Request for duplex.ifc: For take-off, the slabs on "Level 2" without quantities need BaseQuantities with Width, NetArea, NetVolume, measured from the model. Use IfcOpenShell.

First a look at what the model holds.

```python
import ifcopenshell
import ifcopenshell.util.element
import ifcopenshell.util.unit

model = ifcopenshell.open("duplex.ifc")
print(model.schema)
for unit_type in ("LENGTHUNIT", "AREAUNIT", "VOLUMEUNIT"):
    print(unit_type, ifcopenshell.util.unit.calculate_unit_scale(model, unit_type))
storey = next(s for s in model.by_type("IfcBuildingStorey") if s.Name == "Level 2")
slabs = [e for e in ifcopenshell.util.element.get_decomposition(storey) if e.is_a("IfcSlab")]
for e in sorted(slabs, key=lambda e: e.id()):
    print(e.id(), e.is_a(), e.Name, list(ifcopenshell.util.element.get_psets(e, qtos_only=True)), sep=" | ")
```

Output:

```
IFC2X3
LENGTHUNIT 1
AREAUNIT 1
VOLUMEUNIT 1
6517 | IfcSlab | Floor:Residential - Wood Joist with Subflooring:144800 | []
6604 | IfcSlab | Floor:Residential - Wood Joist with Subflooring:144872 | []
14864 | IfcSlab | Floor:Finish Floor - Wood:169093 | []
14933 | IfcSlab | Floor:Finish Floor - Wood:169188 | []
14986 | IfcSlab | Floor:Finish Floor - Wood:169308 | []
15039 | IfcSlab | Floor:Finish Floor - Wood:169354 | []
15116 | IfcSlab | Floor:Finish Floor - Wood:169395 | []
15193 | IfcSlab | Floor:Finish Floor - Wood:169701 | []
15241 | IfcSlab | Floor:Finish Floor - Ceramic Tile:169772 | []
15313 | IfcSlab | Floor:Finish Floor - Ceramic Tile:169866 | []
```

```python
import ifcopenshell
import ifcopenshell.api.pset
import ifcopenshell.geom
import ifcopenshell.util.element
import ifcopenshell.util.shape
import ifcopenshell.util.unit

model = ifcopenshell.open("duplex.ifc")
unit_scale = ifcopenshell.util.unit.calculate_unit_scale(model)
area_scale = ifcopenshell.util.unit.calculate_unit_scale(model, "AREAUNIT")
volume_scale = ifcopenshell.util.unit.calculate_unit_scale(model, "VOLUMEUNIT")
settings = ifcopenshell.geom.settings()

storey = next(s for s in model.by_type("IfcBuildingStorey") if s.Name == "Level 2")
slabs = [e for e in ifcopenshell.util.element.get_decomposition(storey) if e.is_a("IfcSlab")]

for e in sorted(slabs, key=lambda e: e.id()):
    if ifcopenshell.util.element.get_psets(e, qtos_only=True, should_inherit=False):
        continue
    # Geometry comes back in metres, in the element's own axes.
    shape = ifcopenshell.geom.create_shape(settings, e)
    values = {
        "Width": ifcopenshell.util.shape.get_z(shape.geometry) / unit_scale,
        "NetArea": ifcopenshell.util.shape.get_footprint_area(shape.geometry) / area_scale,
        "NetVolume": ifcopenshell.util.shape.get_volume(shape.geometry) / volume_scale,
    }
    qto = ifcopenshell.api.pset.add_qto(model, product=e, name="BaseQuantities")
    ifcopenshell.api.pset.edit_qto(model, qto=qto, properties=values)
    print(e.id(), {k: round(v, 3) for k, v in values.items()})

model.write("duplex_edited.ifc")
```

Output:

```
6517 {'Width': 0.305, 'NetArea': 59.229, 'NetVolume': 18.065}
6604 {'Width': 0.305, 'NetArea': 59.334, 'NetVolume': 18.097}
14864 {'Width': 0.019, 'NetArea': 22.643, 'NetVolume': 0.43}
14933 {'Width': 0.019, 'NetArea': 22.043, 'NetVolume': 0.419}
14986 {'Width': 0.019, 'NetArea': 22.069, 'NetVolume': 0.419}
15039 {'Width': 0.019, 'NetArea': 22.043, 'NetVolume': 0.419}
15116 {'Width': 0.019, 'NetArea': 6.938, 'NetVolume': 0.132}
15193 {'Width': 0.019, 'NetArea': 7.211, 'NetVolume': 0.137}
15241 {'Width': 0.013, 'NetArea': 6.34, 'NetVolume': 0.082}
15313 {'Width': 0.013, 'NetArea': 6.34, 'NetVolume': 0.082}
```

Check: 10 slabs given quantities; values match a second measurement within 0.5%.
